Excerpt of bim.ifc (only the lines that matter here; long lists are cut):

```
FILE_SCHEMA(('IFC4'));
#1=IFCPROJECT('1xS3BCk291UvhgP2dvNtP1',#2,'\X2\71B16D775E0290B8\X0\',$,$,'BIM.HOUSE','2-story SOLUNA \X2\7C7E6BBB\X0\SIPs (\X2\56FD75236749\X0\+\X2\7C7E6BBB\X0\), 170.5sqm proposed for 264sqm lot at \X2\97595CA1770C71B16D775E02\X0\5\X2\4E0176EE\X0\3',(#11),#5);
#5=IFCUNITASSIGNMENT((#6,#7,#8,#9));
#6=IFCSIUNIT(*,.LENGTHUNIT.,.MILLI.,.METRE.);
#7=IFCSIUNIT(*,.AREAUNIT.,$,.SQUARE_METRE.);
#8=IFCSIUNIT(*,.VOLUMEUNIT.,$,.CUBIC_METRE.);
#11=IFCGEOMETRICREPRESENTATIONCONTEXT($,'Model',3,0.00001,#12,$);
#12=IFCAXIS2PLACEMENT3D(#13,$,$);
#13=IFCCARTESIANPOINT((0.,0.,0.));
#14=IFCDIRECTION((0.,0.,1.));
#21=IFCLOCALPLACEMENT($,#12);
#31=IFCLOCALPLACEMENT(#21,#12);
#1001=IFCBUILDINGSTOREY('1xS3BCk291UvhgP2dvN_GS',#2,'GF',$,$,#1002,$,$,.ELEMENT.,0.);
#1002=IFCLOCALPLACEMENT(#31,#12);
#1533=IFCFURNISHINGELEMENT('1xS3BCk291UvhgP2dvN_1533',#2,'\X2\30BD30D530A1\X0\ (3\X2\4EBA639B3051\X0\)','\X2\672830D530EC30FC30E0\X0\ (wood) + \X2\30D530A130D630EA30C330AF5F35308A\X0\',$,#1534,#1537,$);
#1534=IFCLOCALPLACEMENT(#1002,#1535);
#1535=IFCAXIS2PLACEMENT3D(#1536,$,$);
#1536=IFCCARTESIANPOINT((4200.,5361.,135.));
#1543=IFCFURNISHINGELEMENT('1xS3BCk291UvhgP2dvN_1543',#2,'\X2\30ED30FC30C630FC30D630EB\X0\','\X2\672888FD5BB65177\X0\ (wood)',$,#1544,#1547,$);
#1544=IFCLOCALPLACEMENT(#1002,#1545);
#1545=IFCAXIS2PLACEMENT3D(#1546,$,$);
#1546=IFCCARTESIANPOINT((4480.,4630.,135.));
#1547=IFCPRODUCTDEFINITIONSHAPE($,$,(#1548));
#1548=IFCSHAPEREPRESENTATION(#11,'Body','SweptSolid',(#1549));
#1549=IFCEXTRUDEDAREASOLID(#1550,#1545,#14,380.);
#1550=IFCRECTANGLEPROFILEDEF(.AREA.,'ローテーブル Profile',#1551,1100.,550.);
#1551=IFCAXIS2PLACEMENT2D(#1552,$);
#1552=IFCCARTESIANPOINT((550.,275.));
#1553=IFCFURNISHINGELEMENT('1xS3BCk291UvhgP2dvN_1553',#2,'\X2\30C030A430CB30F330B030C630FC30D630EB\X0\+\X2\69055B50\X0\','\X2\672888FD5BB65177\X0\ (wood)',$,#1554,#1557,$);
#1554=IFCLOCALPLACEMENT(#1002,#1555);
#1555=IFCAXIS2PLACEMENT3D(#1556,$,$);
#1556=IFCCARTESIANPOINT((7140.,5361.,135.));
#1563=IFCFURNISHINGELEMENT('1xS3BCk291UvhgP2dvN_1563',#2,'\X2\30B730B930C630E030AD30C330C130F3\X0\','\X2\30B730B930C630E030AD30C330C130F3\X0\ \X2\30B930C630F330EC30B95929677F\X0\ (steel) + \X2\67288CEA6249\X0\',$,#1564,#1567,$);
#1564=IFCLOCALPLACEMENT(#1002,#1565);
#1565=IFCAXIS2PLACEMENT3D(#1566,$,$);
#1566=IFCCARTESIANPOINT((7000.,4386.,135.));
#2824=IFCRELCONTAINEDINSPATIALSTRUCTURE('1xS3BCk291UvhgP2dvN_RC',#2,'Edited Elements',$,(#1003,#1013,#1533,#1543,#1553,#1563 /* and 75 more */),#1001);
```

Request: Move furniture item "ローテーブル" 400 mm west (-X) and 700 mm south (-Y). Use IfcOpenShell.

```python
import ifcopenshell
import ifcopenshell.api.geometry
import ifcopenshell.util.placement
import ifcopenshell.util.unit

model = ifcopenshell.open("bim.ifc")
unit_scale = ifcopenshell.util.unit.calculate_unit_scale(model)

item = model.by_id(1543)
matrix = ifcopenshell.util.placement.get_local_placement(item.ObjectPlacement)
matrix[0, 3] -= 0.4 / unit_scale
matrix[1, 3] -= 0.7 / unit_scale
ifcopenshell.api.geometry.edit_object_placement(model, product=item, matrix=matrix, is_si=False)

print(ifcopenshell.util.placement.get_local_placement(item.ObjectPlacement).round(3) + 0.0)

model.write("bim_v2.ifc")
```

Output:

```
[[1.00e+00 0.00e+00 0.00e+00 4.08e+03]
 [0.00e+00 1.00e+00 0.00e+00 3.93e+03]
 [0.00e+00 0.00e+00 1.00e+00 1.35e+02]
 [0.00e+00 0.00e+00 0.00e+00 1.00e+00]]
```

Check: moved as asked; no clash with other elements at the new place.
